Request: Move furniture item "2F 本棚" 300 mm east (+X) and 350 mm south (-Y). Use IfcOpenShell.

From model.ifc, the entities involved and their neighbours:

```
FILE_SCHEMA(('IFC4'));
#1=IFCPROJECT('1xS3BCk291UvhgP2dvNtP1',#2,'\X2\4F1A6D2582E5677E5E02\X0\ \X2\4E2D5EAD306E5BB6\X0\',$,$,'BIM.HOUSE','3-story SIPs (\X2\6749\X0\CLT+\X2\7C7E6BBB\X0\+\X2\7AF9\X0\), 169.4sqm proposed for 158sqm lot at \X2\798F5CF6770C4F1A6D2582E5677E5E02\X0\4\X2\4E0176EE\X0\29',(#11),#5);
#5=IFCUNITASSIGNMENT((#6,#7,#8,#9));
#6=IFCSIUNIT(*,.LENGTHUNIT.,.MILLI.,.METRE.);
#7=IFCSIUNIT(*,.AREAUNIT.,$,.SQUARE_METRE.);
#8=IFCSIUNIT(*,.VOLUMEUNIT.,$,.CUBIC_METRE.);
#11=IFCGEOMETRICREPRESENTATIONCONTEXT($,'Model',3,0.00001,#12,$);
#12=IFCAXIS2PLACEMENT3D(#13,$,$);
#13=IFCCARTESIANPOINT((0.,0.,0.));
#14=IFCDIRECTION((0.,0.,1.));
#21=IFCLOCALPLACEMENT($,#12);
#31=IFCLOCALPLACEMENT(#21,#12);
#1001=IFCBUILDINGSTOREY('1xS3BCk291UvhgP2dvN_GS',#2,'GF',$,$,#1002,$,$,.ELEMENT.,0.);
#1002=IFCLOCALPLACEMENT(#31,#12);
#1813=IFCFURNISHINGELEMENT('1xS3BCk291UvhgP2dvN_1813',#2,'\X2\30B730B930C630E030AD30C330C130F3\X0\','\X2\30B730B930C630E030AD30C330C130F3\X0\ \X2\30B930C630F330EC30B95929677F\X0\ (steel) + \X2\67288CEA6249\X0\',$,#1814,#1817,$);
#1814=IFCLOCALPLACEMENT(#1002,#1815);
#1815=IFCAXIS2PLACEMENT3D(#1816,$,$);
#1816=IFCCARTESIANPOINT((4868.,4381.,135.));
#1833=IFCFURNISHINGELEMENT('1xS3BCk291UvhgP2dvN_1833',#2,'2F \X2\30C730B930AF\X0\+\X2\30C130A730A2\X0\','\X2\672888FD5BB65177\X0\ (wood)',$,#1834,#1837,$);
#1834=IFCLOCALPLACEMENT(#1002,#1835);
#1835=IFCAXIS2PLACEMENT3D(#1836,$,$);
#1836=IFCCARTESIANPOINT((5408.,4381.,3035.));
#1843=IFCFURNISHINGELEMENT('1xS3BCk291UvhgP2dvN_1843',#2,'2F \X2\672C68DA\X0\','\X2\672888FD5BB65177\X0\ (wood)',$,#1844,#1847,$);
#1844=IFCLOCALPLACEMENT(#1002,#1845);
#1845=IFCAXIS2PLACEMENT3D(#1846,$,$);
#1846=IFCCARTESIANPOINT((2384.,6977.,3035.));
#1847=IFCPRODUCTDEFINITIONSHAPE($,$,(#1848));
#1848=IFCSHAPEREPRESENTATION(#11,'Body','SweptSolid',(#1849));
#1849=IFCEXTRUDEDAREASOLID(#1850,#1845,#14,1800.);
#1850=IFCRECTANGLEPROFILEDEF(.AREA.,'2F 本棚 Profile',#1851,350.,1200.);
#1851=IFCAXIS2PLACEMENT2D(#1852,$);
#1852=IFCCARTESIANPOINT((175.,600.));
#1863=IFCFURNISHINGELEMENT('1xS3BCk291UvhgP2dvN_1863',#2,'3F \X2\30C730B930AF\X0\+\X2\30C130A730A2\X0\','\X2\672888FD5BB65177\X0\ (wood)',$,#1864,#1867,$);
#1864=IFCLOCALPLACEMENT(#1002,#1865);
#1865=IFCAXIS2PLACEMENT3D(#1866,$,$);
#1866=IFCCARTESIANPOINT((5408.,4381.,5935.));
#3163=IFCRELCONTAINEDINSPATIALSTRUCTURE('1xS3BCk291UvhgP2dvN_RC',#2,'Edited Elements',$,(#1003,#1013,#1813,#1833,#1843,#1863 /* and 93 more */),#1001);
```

```python
import ifcopenshell
import ifcopenshell.api.geometry
import ifcopenshell.util.placement

model = ifcopenshell.open("model.ifc")

item = model.by_guid("1xS3BCk291UvhgP2dvN_1843")
matrix = ifcopenshell.util.placement.get_local_placement(item.ObjectPlacement)
matrix[0, 3] += 300.0
matrix[1, 3] -= 350.0
ifcopenshell.api.geometry.edit_object_placement(model, product=item, matrix=matrix, is_si=False)

print(ifcopenshell.util.placement.get_local_placement(item.ObjectPlacement).round(3) + 0.0)

model.write("model_edited.ifc")
```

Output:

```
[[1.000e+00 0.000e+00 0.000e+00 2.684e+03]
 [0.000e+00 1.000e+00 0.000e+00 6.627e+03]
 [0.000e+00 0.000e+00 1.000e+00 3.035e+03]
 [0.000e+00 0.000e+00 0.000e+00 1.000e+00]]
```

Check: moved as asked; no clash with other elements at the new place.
